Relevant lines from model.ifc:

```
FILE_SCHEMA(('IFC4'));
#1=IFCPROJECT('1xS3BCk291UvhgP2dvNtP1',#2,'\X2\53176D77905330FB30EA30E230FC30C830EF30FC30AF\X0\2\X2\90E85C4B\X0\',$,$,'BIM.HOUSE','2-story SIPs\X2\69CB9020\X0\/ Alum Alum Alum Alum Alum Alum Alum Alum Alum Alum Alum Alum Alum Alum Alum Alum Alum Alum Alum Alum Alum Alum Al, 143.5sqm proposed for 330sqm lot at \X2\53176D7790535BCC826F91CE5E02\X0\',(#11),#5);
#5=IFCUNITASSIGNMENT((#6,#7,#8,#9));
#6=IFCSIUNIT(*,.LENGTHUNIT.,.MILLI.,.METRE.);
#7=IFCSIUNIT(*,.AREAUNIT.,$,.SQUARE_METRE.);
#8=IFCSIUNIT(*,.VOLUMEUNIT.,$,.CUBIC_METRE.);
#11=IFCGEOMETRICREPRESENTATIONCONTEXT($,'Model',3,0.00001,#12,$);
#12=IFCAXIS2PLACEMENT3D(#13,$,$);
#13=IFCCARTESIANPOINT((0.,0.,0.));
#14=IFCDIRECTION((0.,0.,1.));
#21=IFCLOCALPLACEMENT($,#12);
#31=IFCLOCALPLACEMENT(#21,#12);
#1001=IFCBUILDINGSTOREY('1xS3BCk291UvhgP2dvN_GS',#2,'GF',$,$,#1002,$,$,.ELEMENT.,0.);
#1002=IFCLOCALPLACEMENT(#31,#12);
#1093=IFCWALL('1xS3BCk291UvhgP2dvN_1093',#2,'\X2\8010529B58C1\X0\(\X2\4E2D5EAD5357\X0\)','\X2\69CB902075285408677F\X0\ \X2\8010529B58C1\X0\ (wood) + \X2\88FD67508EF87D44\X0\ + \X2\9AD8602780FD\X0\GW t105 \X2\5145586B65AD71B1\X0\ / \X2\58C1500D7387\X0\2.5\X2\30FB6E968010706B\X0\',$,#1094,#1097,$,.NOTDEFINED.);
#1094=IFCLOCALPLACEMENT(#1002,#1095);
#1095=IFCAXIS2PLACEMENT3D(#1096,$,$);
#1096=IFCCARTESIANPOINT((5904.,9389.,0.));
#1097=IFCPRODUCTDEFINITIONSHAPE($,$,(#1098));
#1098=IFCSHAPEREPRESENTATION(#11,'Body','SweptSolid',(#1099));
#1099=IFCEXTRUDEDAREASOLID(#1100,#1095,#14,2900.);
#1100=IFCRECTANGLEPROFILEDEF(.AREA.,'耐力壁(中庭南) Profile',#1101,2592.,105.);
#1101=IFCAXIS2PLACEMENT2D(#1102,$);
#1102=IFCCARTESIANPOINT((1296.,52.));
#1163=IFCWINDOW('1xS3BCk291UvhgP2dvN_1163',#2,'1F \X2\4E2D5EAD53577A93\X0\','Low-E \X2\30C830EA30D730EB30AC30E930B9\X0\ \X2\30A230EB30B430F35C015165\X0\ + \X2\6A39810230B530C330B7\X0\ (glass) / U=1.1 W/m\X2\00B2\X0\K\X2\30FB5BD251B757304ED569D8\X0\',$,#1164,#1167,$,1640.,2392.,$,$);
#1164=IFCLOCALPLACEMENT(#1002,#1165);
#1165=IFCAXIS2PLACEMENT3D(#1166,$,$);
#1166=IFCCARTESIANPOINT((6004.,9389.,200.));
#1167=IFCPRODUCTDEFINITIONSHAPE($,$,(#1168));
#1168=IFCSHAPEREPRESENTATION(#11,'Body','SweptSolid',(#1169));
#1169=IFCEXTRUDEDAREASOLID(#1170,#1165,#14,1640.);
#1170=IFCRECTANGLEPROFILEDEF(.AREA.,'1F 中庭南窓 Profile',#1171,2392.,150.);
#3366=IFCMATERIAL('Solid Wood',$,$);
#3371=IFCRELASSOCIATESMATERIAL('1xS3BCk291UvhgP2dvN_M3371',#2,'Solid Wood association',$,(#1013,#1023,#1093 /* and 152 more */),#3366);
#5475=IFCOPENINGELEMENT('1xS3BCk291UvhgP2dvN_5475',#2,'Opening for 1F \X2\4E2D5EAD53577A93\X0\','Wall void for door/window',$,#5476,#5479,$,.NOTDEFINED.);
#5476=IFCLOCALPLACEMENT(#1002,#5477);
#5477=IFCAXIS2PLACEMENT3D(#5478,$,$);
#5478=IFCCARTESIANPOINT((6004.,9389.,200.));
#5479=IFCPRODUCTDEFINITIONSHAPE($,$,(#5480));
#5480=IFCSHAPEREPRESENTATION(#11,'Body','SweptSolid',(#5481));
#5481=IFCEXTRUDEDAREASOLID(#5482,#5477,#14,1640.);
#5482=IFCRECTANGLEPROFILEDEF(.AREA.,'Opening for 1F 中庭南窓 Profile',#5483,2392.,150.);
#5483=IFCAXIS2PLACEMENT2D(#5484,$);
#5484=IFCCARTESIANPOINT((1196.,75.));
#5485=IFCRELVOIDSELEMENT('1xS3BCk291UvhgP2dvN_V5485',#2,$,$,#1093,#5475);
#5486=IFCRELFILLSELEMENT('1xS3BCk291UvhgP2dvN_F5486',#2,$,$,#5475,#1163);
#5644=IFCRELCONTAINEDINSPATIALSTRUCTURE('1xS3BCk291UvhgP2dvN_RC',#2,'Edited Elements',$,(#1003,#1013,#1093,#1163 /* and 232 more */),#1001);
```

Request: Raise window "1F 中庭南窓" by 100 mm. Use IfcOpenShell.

```python
import numpy as np
import ifcopenshell
import ifcopenshell.api.geometry
import ifcopenshell.util.placement
import ifcopenshell.util.unit

model = ifcopenshell.open("model.ifc")
unit_scale = ifcopenshell.util.unit.calculate_unit_scale(model)

window = model.by_guid("1xS3BCk291UvhgP2dvN_1163")
opening = window.FillsVoids[0].RelatingOpeningElement
dz = 100.0

shift = np.array([0.0, 0.0, dz])
# The window is not placed relative to its opening, so move both.
for product in (opening, window):
    matrix = ifcopenshell.util.placement.get_local_placement(product.ObjectPlacement)
    matrix[:3, 3] += shift
    ifcopenshell.api.geometry.edit_object_placement(model, product=product, matrix=matrix, is_si=False)

print(f"moved by {dz * unit_scale:+.3f} m")

model.write("model-out.ifc")
```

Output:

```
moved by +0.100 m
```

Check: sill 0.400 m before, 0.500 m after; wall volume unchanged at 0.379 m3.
